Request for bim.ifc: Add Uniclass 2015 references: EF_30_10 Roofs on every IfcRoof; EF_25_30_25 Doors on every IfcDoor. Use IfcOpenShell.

First a look at what the model holds.

```python
import ifcopenshell

model = ifcopenshell.open("bim.ifc")
print(model.schema)
print("classifications:", [c.Name for c in model.by_type("IfcClassification")])
for ifc_class in ("IfcDoor", "IfcRoof", "IfcStair", "IfcWall", "IfcWindow"):
    print(ifc_class, len(model.by_type(ifc_class)))
```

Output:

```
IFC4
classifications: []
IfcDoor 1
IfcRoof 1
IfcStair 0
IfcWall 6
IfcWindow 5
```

```python
import ifcopenshell
import ifcopenshell.api.classification

model = ifcopenshell.open("bim.ifc")

system = ifcopenshell.api.classification.add_classification(model, classification="Uniclass 2015")

codes = {
    "IfcRoof": ("EF_30_10", "Roofs"),
    "IfcDoor": ("EF_25_30_25", "Doors"),
}
for ifc_class, (code, name) in codes.items():
    products = model.by_type(ifc_class)
    ifcopenshell.api.classification.add_reference(
        model, products=products, classification=system, identification=code, name=name
    )
    print(code, len(products))

model.write("bim-out.ifc")
```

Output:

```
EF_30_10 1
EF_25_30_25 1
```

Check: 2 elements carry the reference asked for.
